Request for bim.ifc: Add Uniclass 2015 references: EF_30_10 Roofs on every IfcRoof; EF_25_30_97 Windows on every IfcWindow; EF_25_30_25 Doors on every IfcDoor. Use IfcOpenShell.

First a look at what the model holds.

```python
import ifcopenshell

model = ifcopenshell.open("bim.ifc")
print(model.schema)
print("classifications:", [c.Name for c in model.by_type("IfcClassification")])
for ifc_class in ("IfcDoor", "IfcRoof", "IfcStair", "IfcWall", "IfcWindow"):
    print(ifc_class, len(model.by_type(ifc_class)))
```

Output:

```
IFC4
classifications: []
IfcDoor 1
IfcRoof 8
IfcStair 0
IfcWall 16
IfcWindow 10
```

```python
import ifcopenshell
import ifcopenshell.api.classification

model = ifcopenshell.open("bim.ifc")

system = ifcopenshell.api.classification.add_classification(model, classification="Uniclass 2015")

codes = {
    "IfcRoof": ("EF_30_10", "Roofs"),
    "IfcWindow": ("EF_25_30_97", "Windows"),
    "IfcDoor": ("EF_25_30_25", "Doors"),
}
for ifc_class, (code, name) in codes.items():
    products = model.by_type(ifc_class)
    ifcopenshell.api.classification.add_reference(
        model, products=products, classification=system, identification=code, name=name
    )
    print(code, len(products))

model.write("bim_updated.ifc")
```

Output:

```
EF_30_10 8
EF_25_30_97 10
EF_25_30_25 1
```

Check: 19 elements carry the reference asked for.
